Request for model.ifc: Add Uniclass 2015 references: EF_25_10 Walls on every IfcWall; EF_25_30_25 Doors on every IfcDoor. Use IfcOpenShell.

First a look at what the model holds.

```python
import ifcopenshell

model = ifcopenshell.open("model.ifc")
print(model.schema)
print("classifications:", [c.Name for c in model.by_type("IfcClassification")])
for ifc_class in ("IfcDoor", "IfcRoof", "IfcStair", "IfcWall", "IfcWindow"):
    print(ifc_class, len(model.by_type(ifc_class)))
```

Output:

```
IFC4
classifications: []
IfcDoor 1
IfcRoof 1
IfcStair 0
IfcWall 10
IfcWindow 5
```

```python
import ifcopenshell
import ifcopenshell.api.classification

model = ifcopenshell.open("model.ifc")

system = ifcopenshell.api.classification.add_classification(model, classification="Uniclass 2015")

codes = {
    "IfcWall": ("EF_25_10", "Walls"),
    "IfcDoor": ("EF_25_30_25", "Doors"),
}
for ifc_class, (code, name) in codes.items():
    products = model.by_type(ifc_class)
    ifcopenshell.api.classification.add_reference(
        model, products=products, classification=system, identification=code, name=name
    )
    print(code, len(products))

model.write("model_rev.ifc")
```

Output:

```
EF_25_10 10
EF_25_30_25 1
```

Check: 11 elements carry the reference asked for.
